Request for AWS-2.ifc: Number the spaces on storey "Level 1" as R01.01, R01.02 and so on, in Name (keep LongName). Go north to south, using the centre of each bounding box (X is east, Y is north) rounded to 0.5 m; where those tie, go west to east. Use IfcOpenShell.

First a look at what the model holds.

```python
import ifcopenshell
import ifcopenshell.util.element
import ifcopenshell.util.placement

model = ifcopenshell.open("AWS-2.ifc")
print(model.schema)
storey = next(s for s in model.by_type("IfcBuildingStorey") if s.Name == "Level 1")
spaces = [e for e in ifcopenshell.util.element.get_decomposition(storey) if e.is_a("IfcSpace")]
for e in sorted(spaces, key=lambda e: e.id()):
    origin = ifcopenshell.util.placement.get_local_placement(e.ObjectPlacement)[:3, 3]
    print(e.id(), e.Name, e.LongName, origin.round(2) + 0.0, sep=" | ")
```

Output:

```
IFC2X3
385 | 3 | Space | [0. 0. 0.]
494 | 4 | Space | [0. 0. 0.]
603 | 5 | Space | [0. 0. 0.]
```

```python
import ifcopenshell
import ifcopenshell.geom
import ifcopenshell.util.element
import ifcopenshell.util.shape

model = ifcopenshell.open("AWS-2.ifc")
settings = ifcopenshell.geom.settings()
settings.set("use-world-coords", True)


def centre(element):
    shape = ifcopenshell.geom.create_shape(settings, element)
    return ifcopenshell.util.shape.get_bbox_centroid(shape.geometry)


storey = next(s for s in model.by_type("IfcBuildingStorey") if s.Name == "Level 1")
spaces = [e for e in ifcopenshell.util.element.get_decomposition(storey) if e.is_a("IfcSpace")]

# Insertion points can sit at a corner or the storey origin, so sort by the geometry (in metres).
centres = {e: centre(e) for e in spaces}
spaces.sort(key=lambda e: (-round(centres[e][1] / 0.5), centres[e][0]))

for i, e in enumerate(spaces, start=1):
    number = f"R01.{i:02d}"
    e.Name = number
    print(e.id(), number)

model.write("AWS-2-out.ifc")
```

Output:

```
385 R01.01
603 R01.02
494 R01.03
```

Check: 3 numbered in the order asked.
